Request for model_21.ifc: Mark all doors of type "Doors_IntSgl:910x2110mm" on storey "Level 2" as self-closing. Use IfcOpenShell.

First a look at what the model holds.

```python
import ifcopenshell
import ifcopenshell.util.element

model = ifcopenshell.open("model_21.ifc")
print(model.schema)
storey = next(s for s in model.by_type("IfcBuildingStorey") if s.Name == "Level 2")
doors = [e for e in ifcopenshell.util.element.get_decomposition(storey) if e.is_a("IfcDoor")]
seen = {}
for e in doors:
    element_type = ifcopenshell.util.element.get_type(e)
    key = (element_type.Name if element_type != e and element_type else None, ifcopenshell.util.element.get_pset(e, "Pset_DoorCommon", "SelfClosing"))
    seen[key] = seen.get(key, 0) + 1
for (name, value), count in sorted(seen.items(), key=str):
    print(count, "x", name, "|", value)
```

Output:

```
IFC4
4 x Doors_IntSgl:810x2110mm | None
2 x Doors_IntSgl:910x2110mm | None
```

```python
import ifcopenshell
import ifcopenshell.api.pset
import ifcopenshell.util.element

model = ifcopenshell.open("model_21.ifc")

storey = next(s for s in model.by_type("IfcBuildingStorey") if s.Name == "Level 2")
doors = [e for e in ifcopenshell.util.element.get_decomposition(storey) if e.is_a("IfcDoor")]

count = 0
for e in doors:
    element_type = ifcopenshell.util.element.get_type(e)
    if element_type in (None, e) or element_type.Name != "Doors_IntSgl:910x2110mm":
        continue
    # add_pset returns the element's existing set when there is one.
    pset = ifcopenshell.api.pset.add_pset(model, product=e, name="Pset_DoorCommon")
    ifcopenshell.api.pset.edit_pset(model, pset=pset, properties={"SelfClosing": True})
    count += 1

print(count, "doors updated")

model.write("model_21-out.ifc")
```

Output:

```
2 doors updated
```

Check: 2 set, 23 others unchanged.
